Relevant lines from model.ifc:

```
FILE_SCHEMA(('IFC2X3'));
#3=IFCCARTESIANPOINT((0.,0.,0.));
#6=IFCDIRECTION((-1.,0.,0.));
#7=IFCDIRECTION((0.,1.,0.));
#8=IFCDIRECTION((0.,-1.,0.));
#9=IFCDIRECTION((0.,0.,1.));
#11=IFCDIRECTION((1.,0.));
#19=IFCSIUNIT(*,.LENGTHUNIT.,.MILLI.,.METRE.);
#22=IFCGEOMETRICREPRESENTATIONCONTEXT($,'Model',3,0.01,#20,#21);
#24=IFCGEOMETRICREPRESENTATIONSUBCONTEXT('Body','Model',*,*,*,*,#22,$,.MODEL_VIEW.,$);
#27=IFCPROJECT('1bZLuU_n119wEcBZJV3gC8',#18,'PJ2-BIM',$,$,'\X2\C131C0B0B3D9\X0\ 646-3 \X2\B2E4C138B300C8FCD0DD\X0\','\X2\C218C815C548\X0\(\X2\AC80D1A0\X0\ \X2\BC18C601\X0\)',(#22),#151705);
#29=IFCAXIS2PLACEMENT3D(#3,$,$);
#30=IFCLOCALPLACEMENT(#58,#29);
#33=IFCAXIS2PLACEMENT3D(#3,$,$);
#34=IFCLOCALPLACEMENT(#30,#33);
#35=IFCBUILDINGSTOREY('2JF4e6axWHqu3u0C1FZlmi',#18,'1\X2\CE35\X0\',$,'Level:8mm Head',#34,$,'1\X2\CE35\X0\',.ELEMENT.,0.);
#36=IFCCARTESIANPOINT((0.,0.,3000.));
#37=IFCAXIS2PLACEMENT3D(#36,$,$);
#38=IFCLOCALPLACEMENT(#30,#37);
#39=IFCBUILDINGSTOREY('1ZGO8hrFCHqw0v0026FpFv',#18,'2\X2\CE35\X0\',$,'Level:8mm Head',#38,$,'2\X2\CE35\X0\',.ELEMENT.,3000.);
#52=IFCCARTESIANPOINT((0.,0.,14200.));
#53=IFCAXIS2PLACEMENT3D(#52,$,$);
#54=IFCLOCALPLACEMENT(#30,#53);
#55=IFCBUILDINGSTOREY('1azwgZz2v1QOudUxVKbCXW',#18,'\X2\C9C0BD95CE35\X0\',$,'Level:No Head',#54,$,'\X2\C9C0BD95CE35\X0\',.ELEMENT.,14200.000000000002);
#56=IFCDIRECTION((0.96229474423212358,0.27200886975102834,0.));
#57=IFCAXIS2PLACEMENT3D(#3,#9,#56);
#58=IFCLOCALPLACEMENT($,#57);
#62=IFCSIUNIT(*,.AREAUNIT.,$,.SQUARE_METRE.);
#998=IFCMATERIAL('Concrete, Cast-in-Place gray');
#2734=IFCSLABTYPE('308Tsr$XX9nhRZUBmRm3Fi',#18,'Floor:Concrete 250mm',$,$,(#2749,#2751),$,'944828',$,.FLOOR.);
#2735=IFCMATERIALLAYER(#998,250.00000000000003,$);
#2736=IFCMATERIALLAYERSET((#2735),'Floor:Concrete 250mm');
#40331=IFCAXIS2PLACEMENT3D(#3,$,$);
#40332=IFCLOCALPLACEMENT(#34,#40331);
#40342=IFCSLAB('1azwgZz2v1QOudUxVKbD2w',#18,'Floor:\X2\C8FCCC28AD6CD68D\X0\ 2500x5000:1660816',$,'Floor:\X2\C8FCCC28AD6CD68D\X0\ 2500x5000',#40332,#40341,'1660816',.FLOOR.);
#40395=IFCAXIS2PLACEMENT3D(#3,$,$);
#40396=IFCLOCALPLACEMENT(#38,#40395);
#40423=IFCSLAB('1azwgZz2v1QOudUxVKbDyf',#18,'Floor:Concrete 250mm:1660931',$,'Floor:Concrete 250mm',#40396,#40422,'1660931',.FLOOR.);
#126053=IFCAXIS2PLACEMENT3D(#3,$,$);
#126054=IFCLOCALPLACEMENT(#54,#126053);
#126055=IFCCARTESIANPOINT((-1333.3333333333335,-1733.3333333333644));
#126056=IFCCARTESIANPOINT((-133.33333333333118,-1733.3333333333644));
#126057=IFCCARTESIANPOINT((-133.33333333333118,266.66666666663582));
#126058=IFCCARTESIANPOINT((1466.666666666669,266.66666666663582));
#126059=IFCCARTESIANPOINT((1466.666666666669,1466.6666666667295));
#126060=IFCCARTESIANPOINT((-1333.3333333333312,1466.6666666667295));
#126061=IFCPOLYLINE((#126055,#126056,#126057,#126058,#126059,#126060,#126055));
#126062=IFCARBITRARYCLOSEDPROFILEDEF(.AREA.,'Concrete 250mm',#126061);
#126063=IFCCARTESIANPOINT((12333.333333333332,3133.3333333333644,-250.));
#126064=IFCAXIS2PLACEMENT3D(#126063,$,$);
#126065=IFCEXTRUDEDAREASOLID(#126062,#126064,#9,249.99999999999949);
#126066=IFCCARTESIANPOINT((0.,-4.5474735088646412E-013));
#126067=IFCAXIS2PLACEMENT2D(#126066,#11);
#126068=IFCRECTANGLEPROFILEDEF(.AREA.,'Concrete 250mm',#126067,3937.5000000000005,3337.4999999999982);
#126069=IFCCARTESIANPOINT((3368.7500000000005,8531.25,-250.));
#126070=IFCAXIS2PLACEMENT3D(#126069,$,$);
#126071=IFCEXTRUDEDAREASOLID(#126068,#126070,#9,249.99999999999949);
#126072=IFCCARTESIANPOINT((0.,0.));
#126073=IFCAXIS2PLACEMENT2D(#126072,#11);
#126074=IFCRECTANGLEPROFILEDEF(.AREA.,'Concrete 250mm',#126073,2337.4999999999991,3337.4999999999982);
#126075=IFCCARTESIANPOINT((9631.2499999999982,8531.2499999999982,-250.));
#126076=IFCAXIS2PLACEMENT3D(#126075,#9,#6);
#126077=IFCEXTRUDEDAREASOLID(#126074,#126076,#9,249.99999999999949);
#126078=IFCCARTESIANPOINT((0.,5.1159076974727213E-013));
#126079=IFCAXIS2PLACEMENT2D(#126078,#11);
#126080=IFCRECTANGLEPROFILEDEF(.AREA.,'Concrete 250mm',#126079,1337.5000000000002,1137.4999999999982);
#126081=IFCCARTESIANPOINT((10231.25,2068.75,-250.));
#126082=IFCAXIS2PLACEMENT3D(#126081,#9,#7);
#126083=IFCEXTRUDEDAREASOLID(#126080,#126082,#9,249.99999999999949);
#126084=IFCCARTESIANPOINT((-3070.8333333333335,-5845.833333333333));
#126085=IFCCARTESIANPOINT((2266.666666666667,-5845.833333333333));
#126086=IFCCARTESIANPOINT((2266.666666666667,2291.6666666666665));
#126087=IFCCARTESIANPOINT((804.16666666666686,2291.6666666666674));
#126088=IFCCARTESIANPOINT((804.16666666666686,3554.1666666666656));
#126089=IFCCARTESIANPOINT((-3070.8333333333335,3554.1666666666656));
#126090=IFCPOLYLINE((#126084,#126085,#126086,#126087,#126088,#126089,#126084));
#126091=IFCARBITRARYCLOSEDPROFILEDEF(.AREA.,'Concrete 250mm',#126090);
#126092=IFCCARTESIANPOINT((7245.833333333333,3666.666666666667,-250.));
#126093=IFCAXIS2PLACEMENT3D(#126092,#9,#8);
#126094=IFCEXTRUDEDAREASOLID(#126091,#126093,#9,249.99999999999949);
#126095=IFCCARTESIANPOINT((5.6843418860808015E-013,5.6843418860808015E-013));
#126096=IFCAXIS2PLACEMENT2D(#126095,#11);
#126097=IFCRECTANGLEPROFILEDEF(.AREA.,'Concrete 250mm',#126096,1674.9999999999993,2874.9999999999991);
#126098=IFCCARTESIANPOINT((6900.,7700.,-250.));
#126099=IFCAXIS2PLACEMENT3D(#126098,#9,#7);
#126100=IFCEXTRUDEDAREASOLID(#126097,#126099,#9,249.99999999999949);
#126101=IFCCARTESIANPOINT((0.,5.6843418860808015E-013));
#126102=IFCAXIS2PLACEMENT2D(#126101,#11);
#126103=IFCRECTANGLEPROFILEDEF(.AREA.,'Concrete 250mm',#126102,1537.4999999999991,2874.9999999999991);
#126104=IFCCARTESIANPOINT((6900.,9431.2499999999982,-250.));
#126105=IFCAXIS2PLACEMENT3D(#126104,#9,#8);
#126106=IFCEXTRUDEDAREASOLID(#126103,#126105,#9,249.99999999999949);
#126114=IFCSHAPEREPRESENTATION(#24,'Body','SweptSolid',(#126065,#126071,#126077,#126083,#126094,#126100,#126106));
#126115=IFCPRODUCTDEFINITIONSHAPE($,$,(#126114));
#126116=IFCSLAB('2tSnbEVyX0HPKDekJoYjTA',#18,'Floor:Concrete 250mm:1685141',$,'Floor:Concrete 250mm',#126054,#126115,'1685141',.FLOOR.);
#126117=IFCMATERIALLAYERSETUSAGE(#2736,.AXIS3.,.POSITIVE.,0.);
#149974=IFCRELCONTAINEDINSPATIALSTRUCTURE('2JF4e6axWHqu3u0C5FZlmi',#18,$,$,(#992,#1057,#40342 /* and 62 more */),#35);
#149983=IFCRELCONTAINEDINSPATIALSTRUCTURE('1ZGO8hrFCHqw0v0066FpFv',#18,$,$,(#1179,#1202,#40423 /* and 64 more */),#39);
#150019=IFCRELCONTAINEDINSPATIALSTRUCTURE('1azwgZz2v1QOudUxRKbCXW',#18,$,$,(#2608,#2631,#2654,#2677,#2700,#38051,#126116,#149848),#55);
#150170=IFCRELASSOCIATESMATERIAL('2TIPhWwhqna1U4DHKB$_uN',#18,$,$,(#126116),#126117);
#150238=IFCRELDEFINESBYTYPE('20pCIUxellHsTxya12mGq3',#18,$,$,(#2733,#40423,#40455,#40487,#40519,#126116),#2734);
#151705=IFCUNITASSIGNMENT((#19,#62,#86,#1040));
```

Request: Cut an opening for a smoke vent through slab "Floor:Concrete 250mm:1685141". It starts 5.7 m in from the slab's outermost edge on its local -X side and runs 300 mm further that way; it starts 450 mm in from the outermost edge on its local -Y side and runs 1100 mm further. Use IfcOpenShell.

```python
import numpy as np
import ifcopenshell
import ifcopenshell.api.feature
import ifcopenshell.api.geometry
import ifcopenshell.api.root
import ifcopenshell.geom
import ifcopenshell.util.placement
import ifcopenshell.util.representation
import ifcopenshell.util.shape
import ifcopenshell.util.unit

model = ifcopenshell.open("model.ifc")
unit_scale = ifcopenshell.util.unit.calculate_unit_scale(model)
settings = ifcopenshell.geom.settings()


def volume(element):
    """Net volume in cubic metres, openings subtracted."""
    shape = ifcopenshell.geom.create_shape(settings, element)
    return ifcopenshell.util.shape.get_volume(shape.geometry)


slab = model.by_guid("2tSnbEVyX0HPKDekJoYjTA")
before = volume(slab)

# Extent in the slab's own axes, in metres. The edges named are its -X and -Y sides.
slab_shape = ifcopenshell.geom.create_shape(settings, slab)
vertices = ifcopenshell.util.shape.get_vertices(slab_shape.geometry)
x_min, y_min, bottom = vertices.min(axis=0)
top = vertices[:, 2].max()

opening = ifcopenshell.api.root.create_entity(model, ifc_class="IfcOpeningElement", name="Smoke vent opening")
context = ifcopenshell.util.representation.get_context(model, "Model", "Body", "MODEL_VIEW")
width, depth = 0.3, 1.1
outline = [(0.0, 0.0), (width, 0.0), (width, depth), (0.0, depth), (0.0, 0.0)]
# Overshoot both faces by 50 mm so the cut is clean.
shape = ifcopenshell.api.geometry.add_slab_representation(
    model, context=context, depth=top - bottom + 0.1, polyline=outline
)
ifcopenshell.api.geometry.assign_representation(model, product=opening, representation=shape)

matrix = ifcopenshell.util.placement.get_local_placement(slab.ObjectPlacement)
matrix[:, 3] = matrix @ np.append(np.array([x_min + 5.7, y_min + 0.45, bottom - 0.05]) / unit_scale, 1.0)
ifcopenshell.api.geometry.edit_object_placement(model, product=opening, matrix=matrix, is_si=False)
ifcopenshell.api.feature.add_feature(model, feature=opening, element=slab)

after = volume(slab)

print(f"slab volume {before:.3f} -> {after:.3f} m3")

model.write("model_v2.ifc")
```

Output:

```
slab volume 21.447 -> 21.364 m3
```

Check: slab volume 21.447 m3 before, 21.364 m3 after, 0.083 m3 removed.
